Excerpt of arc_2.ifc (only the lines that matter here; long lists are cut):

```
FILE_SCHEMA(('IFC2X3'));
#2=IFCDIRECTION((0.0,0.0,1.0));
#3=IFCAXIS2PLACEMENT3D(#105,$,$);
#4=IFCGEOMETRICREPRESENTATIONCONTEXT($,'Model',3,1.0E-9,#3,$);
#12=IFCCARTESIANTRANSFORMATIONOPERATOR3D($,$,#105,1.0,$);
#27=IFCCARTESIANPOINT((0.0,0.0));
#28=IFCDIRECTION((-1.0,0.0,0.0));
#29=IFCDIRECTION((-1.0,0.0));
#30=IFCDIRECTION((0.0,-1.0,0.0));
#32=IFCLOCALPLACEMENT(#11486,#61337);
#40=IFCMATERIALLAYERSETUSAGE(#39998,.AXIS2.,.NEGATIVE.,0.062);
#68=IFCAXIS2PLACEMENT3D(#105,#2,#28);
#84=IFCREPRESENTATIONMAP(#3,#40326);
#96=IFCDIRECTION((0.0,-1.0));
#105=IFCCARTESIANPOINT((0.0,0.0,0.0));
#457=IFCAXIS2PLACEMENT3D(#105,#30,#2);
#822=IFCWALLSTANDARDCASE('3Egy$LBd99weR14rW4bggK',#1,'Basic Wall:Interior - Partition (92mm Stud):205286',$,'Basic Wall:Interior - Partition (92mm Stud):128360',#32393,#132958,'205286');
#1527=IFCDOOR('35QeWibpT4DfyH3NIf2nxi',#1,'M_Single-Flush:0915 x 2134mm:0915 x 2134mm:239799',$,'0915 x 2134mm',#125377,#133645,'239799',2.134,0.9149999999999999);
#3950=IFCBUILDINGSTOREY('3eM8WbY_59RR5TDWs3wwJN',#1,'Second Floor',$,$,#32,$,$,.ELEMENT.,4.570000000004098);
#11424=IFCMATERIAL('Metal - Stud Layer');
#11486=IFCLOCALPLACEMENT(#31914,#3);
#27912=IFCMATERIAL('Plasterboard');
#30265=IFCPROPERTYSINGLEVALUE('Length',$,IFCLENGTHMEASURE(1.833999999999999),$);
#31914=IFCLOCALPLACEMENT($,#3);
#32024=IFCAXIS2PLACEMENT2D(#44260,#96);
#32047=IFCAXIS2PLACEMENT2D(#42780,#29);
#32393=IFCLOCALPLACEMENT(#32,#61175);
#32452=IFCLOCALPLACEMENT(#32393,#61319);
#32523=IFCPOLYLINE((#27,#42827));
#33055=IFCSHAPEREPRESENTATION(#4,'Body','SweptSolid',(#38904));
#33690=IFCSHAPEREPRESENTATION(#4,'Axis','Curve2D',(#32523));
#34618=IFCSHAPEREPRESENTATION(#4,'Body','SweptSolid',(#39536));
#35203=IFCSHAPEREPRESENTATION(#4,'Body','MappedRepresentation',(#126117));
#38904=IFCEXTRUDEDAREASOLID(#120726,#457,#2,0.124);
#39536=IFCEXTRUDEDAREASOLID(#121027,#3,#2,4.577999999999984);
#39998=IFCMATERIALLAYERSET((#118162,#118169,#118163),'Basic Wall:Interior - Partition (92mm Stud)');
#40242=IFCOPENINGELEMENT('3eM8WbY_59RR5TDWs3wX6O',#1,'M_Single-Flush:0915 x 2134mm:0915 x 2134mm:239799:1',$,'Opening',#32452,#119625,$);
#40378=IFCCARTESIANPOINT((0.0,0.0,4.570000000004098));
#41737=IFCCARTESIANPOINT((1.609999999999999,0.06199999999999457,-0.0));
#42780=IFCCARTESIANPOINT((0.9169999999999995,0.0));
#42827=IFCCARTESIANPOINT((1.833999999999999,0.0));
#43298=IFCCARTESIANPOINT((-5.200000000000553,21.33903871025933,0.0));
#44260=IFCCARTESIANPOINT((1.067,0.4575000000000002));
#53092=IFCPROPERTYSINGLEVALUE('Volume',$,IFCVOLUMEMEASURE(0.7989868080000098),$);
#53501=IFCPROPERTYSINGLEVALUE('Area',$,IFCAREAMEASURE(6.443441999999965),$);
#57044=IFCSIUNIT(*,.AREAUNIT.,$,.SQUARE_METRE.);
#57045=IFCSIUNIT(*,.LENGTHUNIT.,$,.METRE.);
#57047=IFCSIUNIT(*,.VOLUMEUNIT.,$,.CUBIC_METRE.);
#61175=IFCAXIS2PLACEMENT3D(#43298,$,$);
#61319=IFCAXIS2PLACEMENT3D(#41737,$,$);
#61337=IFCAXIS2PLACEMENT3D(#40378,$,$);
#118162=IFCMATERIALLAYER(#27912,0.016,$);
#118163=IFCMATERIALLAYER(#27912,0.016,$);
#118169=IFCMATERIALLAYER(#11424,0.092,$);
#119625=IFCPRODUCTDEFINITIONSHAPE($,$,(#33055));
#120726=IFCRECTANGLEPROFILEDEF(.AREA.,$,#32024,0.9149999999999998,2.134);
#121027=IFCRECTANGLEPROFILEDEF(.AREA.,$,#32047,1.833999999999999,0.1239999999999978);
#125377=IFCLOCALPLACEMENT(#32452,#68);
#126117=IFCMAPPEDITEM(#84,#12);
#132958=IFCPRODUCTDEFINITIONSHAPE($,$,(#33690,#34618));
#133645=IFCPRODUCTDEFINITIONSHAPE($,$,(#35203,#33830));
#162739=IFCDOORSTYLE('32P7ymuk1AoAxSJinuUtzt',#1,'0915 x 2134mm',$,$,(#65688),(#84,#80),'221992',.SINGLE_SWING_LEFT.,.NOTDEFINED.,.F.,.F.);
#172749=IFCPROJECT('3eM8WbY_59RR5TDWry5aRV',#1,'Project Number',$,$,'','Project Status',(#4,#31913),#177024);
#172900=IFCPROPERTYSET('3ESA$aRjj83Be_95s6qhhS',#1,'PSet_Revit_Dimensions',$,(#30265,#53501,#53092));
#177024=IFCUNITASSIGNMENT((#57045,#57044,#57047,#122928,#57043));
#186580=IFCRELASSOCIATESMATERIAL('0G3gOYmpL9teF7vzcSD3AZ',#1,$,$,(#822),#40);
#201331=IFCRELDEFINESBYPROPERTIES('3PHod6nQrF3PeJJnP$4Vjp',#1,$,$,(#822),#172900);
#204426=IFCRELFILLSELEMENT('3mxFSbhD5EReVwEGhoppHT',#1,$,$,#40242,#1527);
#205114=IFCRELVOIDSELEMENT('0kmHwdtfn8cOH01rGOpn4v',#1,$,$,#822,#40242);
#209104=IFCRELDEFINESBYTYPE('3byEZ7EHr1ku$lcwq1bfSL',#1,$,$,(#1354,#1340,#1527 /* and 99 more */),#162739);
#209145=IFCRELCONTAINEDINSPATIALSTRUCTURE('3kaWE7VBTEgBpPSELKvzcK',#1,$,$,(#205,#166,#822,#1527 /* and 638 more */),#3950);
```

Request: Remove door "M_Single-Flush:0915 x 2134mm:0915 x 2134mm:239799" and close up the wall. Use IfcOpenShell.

```python
import ifcopenshell
import ifcopenshell.api.feature
import ifcopenshell.api.pset
import ifcopenshell.api.root
import ifcopenshell.geom
import ifcopenshell.util.element
import ifcopenshell.util.shape
import ifcopenshell.util.unit

model = ifcopenshell.open("arc_2.ifc")
area_scale = ifcopenshell.util.unit.calculate_unit_scale(model, "AREAUNIT")
volume_scale = ifcopenshell.util.unit.calculate_unit_scale(model, "VOLUMEUNIT")
settings = ifcopenshell.geom.settings()


def volume(element):
    """Net volume in cubic metres, openings subtracted."""
    shape = ifcopenshell.geom.create_shape(settings, element)
    return ifcopenshell.util.shape.get_volume(shape.geometry)


door = model.by_guid("35QeWibpT4DfyH3NIf2nxi")
opening = door.FillsVoids[0].RelatingOpeningElement
wall = opening.VoidsElements[0].RelatingBuildingElement
before = volume(wall)

ifcopenshell.api.root.remove_product(model, product=door)
ifcopenshell.api.feature.remove_feature(model, feature=opening)

after = volume(wall)
thickness = 0.124  # wall thickness in metres

# Update the wall's stored quantities.
pset = model.by_id(ifcopenshell.util.element.get_pset(wall, "PSet_Revit_Dimensions", should_inherit=False)["id"])
ifcopenshell.api.pset.edit_pset(model, pset=pset, properties={
    "Area": model.create_entity("IfcAreaMeasure", after / thickness / area_scale),
    "Volume": model.create_entity("IfcVolumeMeasure", after / volume_scale),
})

print(f"wall volume {before:.3f} -> {after:.3f} m3")

model.write("arc_2_rev.ifc")
```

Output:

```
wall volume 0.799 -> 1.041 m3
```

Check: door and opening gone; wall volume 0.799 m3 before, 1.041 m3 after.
